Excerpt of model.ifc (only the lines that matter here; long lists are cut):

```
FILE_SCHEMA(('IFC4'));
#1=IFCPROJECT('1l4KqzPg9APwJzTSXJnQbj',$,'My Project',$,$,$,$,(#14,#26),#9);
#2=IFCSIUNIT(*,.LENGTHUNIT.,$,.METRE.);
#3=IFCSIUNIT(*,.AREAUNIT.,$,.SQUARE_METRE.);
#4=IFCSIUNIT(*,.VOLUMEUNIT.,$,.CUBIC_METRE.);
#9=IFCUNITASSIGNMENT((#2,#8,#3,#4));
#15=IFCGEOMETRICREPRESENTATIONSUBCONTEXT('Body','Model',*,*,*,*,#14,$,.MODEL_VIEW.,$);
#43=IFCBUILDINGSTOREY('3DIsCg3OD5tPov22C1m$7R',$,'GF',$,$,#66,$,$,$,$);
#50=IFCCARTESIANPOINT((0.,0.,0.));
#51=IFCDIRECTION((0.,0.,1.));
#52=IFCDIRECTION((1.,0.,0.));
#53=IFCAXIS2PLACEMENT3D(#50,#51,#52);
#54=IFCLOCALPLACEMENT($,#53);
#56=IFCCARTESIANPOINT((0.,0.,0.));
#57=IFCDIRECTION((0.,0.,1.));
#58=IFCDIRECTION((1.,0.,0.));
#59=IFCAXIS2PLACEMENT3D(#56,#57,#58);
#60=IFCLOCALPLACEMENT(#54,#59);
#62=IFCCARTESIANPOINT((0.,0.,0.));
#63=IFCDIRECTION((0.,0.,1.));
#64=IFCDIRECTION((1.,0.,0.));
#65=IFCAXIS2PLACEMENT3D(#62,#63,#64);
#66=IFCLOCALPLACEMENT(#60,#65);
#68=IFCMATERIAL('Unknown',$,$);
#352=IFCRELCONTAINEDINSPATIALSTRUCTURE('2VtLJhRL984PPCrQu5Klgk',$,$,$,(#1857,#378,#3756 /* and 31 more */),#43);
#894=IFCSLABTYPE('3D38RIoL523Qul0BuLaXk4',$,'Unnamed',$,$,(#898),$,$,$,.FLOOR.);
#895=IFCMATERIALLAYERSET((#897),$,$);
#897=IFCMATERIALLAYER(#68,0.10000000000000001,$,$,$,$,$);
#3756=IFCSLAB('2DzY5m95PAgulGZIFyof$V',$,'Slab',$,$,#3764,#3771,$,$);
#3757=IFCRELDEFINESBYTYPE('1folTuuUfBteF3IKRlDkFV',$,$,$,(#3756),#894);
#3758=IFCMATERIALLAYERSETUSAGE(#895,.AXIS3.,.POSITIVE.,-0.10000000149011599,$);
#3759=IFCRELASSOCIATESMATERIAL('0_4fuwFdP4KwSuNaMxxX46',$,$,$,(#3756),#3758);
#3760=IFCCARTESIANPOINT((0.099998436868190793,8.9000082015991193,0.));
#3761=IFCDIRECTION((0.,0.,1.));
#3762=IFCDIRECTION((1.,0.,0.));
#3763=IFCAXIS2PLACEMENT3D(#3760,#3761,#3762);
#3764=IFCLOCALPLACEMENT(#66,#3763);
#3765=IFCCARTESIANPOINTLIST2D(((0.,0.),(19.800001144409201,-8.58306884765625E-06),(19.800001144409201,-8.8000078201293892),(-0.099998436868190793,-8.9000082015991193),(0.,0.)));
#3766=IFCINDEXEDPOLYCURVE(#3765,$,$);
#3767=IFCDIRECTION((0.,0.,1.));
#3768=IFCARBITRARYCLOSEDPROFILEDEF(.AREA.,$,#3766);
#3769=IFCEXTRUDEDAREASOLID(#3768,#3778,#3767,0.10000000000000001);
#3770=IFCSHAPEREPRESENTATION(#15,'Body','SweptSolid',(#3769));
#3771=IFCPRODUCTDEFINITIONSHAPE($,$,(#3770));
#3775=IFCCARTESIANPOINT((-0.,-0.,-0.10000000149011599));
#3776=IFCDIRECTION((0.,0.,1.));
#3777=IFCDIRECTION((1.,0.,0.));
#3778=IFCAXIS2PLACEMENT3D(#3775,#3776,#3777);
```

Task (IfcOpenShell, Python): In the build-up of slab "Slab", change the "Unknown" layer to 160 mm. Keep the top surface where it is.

```python
import ifcopenshell
import ifcopenshell.util.element
import ifcopenshell.util.representation
import ifcopenshell.util.unit

model = ifcopenshell.open("model.ifc")
unit_scale = ifcopenshell.util.unit.calculate_unit_scale(model)

layer_set = model.by_id(895)
layer = next(l for l in layer_set.MaterialLayers if l.Material and l.Material.Name == "Unknown")
change = 0.16 / unit_scale - layer.LayerThickness
layer.LayerThickness += change

# Geometry does not follow the layer set by itself.
slabs = [e for e in ifcopenshell.util.element.get_elements_by_material(model, layer_set) if e.is_a("IfcSlab")]
for slab in sorted(slabs, key=lambda e: e.id()):
    body = ifcopenshell.util.representation.get_representation(slab, "Model", "Body")
    solid = body.Items[0]
    old_depth = solid.Depth
    solid.Depth += change
    # Extruded upwards: lower the start of the extrusion so the top stays.
    x, y, z = solid.Position.Location.Coordinates
    solid.Position.Location = model.createIfcCartesianPoint((x, y, z - change))
    print(slab.id(), f"{old_depth:g} -> {solid.Depth:g}")

# The layers are counted up from the underside, which has moved.
for usage in {ifcopenshell.util.element.get_material(slab) for slab in slabs}:
    usage.OffsetFromReferenceLine -= change

model.write("model_v2.ifc")
```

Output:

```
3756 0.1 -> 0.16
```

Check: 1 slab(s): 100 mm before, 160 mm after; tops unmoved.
